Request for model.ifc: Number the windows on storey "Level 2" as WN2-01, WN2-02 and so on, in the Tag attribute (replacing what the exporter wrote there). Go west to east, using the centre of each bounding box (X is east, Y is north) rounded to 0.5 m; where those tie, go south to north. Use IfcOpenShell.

First a look at what the model holds.

```python
import ifcopenshell
import ifcopenshell.util.element
import ifcopenshell.util.placement

model = ifcopenshell.open("model.ifc")
print(model.schema)
storey = next(s for s in model.by_type("IfcBuildingStorey") if s.Name == "Level 2")
windows = [e for e in ifcopenshell.util.element.get_decomposition(storey) if e.is_a("IfcWindow")]
for e in sorted(windows, key=lambda e: e.id()):
    origin = ifcopenshell.util.placement.get_local_placement(e.ObjectPlacement)[:3, 3]
    print(e.id(), e.Tag, e.Name, origin.round(2) + 0.0, sep=" | ")
```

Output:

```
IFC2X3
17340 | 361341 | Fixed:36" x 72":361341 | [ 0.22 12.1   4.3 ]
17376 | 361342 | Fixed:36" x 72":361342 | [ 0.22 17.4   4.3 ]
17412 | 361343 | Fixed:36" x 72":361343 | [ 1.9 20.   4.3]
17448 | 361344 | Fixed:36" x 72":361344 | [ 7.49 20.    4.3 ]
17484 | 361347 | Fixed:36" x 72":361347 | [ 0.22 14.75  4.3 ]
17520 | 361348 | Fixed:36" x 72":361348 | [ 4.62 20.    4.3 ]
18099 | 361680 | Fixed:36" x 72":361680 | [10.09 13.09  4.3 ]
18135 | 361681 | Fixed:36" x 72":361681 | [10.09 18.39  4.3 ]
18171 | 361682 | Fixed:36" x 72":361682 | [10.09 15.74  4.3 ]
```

```python
import ifcopenshell
import ifcopenshell.geom
import ifcopenshell.util.element
import ifcopenshell.util.shape

model = ifcopenshell.open("model.ifc")
settings = ifcopenshell.geom.settings()
settings.set("use-world-coords", True)


def centre(element):
    shape = ifcopenshell.geom.create_shape(settings, element)
    return ifcopenshell.util.shape.get_bbox_centroid(shape.geometry)


storey = next(s for s in model.by_type("IfcBuildingStorey") if s.Name == "Level 2")
windows = [e for e in ifcopenshell.util.element.get_decomposition(storey) if e.is_a("IfcWindow")]

# Insertion points can sit at a corner or the storey origin, so sort by the geometry (in metres).
centres = {e: centre(e) for e in windows}
windows.sort(key=lambda e: (round(centres[e][0] / 0.5), centres[e][1]))

for i, e in enumerate(windows, start=1):
    number = f"WN2-{i:02d}"
    e.Tag = number
    print(e.id(), number)

model.write("model-out.ifc")
```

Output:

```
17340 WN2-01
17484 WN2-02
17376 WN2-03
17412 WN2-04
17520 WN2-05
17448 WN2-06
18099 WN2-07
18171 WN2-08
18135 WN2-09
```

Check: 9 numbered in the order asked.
